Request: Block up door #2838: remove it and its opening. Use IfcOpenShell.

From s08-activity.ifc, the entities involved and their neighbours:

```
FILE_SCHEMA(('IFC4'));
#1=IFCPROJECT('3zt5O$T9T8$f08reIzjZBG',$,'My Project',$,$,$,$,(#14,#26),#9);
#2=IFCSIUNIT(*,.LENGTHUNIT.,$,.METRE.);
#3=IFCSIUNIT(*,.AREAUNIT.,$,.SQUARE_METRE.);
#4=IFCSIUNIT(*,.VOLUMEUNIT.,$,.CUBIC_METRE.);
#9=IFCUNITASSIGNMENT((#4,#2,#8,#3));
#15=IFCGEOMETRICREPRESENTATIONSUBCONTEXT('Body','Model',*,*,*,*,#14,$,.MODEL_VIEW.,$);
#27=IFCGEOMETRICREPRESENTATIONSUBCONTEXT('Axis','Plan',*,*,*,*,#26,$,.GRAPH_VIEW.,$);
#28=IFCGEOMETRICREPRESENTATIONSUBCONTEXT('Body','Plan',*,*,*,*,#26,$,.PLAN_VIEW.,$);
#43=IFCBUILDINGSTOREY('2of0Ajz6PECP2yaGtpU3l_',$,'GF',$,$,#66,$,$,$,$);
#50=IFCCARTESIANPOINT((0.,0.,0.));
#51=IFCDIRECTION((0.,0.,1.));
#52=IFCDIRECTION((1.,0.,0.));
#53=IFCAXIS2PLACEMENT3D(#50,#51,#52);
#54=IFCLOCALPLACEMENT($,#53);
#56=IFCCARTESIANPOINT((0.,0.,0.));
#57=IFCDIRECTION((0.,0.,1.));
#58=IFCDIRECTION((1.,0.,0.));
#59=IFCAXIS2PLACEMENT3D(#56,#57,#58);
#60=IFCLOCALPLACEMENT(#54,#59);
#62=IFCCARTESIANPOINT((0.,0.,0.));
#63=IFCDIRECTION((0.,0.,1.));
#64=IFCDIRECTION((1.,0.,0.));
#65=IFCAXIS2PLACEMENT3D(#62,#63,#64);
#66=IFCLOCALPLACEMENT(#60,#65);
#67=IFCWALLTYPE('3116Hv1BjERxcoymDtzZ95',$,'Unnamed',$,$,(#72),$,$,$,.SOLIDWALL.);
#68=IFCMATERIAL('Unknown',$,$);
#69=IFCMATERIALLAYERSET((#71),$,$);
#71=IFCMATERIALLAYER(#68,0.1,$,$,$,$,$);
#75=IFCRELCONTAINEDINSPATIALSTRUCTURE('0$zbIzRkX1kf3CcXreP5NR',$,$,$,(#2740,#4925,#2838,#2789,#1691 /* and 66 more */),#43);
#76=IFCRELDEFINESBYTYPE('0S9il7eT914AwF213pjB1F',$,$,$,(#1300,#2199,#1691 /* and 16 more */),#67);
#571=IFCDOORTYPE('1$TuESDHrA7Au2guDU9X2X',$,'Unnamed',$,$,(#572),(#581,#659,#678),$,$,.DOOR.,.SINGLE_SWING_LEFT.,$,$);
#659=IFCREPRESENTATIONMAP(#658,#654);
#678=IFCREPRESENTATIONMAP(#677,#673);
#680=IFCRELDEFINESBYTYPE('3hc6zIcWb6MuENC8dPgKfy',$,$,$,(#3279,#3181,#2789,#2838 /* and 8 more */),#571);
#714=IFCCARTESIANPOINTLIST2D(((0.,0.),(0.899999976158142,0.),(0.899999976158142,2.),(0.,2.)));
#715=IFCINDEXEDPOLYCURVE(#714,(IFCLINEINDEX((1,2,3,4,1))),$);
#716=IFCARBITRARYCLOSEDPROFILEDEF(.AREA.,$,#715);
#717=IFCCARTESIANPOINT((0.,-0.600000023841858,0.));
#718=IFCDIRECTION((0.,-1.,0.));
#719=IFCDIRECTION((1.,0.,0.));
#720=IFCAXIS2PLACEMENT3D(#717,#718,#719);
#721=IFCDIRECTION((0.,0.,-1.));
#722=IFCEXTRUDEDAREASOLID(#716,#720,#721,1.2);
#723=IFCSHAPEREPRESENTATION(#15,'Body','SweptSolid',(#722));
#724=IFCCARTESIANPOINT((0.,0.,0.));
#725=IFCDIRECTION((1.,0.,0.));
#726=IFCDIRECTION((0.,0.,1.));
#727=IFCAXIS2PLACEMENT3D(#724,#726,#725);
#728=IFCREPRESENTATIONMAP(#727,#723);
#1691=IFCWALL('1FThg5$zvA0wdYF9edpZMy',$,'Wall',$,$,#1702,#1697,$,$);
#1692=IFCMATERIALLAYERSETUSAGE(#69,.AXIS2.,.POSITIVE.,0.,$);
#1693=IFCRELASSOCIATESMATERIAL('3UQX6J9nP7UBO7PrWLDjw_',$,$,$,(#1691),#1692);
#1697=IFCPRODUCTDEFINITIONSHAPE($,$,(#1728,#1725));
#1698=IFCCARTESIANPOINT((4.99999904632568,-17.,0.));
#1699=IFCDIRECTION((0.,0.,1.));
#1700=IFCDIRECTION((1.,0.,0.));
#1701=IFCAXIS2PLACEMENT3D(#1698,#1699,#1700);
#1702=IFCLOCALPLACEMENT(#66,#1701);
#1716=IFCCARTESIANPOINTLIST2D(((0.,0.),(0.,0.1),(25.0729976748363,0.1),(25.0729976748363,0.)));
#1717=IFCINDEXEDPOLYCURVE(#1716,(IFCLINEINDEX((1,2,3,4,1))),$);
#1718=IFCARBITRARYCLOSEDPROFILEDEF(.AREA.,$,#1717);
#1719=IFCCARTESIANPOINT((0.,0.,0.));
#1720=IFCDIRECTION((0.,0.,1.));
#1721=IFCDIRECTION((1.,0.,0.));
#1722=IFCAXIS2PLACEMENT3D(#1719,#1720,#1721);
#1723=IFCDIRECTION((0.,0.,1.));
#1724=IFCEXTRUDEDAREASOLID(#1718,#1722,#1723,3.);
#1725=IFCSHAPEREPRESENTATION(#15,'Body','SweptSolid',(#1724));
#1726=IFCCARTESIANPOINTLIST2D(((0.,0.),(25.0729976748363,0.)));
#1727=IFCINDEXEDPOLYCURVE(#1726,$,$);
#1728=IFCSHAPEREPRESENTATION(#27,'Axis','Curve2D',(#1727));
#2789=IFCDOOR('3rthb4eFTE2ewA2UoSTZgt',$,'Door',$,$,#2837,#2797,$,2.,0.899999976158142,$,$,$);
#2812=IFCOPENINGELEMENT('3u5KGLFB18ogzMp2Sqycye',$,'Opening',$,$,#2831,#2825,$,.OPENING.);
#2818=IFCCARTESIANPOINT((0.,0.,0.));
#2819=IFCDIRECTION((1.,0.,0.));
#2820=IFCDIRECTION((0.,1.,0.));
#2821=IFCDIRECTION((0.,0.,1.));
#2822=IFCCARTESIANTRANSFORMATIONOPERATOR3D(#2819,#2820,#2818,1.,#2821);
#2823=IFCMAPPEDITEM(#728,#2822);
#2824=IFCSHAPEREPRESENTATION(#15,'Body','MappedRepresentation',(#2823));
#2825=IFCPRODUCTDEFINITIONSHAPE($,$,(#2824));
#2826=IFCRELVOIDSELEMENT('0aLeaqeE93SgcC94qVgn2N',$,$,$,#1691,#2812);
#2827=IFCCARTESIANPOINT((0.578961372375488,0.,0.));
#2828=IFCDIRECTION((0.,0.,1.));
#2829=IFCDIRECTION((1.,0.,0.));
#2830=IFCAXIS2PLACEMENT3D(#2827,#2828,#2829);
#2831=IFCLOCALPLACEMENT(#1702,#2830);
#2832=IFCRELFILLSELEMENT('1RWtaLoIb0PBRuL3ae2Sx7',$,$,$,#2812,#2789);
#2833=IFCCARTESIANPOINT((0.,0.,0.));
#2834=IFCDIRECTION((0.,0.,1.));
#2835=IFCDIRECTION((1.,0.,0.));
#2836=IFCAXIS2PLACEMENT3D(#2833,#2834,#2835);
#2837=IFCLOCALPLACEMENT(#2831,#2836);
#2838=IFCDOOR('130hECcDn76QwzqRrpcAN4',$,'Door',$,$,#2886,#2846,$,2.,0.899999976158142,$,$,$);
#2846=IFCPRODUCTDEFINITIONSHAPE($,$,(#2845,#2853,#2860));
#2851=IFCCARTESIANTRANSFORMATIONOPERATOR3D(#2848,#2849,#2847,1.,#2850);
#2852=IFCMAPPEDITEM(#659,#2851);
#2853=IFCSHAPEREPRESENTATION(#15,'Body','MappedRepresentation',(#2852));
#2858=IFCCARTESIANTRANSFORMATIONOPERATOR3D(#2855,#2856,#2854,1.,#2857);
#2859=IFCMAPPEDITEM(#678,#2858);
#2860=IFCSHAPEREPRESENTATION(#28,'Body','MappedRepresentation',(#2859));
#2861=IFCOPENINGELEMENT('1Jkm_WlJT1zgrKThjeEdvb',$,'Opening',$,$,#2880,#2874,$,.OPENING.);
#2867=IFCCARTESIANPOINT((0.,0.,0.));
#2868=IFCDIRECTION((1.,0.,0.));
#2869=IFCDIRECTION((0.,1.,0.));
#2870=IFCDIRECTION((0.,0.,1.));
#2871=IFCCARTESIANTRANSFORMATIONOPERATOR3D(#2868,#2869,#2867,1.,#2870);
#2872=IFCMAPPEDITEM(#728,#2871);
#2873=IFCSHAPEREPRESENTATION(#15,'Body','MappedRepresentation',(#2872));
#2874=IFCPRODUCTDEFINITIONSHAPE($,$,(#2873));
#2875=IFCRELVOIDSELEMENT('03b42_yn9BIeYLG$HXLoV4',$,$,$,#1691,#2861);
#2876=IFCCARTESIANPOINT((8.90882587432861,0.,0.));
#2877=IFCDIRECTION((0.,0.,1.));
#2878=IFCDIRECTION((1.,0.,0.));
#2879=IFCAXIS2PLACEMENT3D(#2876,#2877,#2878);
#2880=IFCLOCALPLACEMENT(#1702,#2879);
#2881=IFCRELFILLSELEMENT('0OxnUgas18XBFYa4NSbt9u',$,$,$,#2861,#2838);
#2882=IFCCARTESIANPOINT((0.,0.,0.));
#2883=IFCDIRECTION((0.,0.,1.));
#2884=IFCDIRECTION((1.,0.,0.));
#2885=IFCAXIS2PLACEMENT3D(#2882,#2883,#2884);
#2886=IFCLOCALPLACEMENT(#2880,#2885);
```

```python
import ifcopenshell
import ifcopenshell.api.feature
import ifcopenshell.api.root
import ifcopenshell.geom
import ifcopenshell.util.shape

model = ifcopenshell.open("s08-activity.ifc")
settings = ifcopenshell.geom.settings()


def volume(element):
    """Net volume in cubic metres, openings subtracted."""
    shape = ifcopenshell.geom.create_shape(settings, element)
    return ifcopenshell.util.shape.get_volume(shape.geometry)


door = model.by_guid("130hECcDn76QwzqRrpcAN4")
opening = door.FillsVoids[0].RelatingOpeningElement
wall = opening.VoidsElements[0].RelatingBuildingElement
before = volume(wall)

ifcopenshell.api.root.remove_product(model, product=door)
ifcopenshell.api.feature.remove_feature(model, feature=opening)

after = volume(wall)

print(f"wall volume {before:.3f} -> {after:.3f} m3")

model.write("s08-activity-out.ifc")
```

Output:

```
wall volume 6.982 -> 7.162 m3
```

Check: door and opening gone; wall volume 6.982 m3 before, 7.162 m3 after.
